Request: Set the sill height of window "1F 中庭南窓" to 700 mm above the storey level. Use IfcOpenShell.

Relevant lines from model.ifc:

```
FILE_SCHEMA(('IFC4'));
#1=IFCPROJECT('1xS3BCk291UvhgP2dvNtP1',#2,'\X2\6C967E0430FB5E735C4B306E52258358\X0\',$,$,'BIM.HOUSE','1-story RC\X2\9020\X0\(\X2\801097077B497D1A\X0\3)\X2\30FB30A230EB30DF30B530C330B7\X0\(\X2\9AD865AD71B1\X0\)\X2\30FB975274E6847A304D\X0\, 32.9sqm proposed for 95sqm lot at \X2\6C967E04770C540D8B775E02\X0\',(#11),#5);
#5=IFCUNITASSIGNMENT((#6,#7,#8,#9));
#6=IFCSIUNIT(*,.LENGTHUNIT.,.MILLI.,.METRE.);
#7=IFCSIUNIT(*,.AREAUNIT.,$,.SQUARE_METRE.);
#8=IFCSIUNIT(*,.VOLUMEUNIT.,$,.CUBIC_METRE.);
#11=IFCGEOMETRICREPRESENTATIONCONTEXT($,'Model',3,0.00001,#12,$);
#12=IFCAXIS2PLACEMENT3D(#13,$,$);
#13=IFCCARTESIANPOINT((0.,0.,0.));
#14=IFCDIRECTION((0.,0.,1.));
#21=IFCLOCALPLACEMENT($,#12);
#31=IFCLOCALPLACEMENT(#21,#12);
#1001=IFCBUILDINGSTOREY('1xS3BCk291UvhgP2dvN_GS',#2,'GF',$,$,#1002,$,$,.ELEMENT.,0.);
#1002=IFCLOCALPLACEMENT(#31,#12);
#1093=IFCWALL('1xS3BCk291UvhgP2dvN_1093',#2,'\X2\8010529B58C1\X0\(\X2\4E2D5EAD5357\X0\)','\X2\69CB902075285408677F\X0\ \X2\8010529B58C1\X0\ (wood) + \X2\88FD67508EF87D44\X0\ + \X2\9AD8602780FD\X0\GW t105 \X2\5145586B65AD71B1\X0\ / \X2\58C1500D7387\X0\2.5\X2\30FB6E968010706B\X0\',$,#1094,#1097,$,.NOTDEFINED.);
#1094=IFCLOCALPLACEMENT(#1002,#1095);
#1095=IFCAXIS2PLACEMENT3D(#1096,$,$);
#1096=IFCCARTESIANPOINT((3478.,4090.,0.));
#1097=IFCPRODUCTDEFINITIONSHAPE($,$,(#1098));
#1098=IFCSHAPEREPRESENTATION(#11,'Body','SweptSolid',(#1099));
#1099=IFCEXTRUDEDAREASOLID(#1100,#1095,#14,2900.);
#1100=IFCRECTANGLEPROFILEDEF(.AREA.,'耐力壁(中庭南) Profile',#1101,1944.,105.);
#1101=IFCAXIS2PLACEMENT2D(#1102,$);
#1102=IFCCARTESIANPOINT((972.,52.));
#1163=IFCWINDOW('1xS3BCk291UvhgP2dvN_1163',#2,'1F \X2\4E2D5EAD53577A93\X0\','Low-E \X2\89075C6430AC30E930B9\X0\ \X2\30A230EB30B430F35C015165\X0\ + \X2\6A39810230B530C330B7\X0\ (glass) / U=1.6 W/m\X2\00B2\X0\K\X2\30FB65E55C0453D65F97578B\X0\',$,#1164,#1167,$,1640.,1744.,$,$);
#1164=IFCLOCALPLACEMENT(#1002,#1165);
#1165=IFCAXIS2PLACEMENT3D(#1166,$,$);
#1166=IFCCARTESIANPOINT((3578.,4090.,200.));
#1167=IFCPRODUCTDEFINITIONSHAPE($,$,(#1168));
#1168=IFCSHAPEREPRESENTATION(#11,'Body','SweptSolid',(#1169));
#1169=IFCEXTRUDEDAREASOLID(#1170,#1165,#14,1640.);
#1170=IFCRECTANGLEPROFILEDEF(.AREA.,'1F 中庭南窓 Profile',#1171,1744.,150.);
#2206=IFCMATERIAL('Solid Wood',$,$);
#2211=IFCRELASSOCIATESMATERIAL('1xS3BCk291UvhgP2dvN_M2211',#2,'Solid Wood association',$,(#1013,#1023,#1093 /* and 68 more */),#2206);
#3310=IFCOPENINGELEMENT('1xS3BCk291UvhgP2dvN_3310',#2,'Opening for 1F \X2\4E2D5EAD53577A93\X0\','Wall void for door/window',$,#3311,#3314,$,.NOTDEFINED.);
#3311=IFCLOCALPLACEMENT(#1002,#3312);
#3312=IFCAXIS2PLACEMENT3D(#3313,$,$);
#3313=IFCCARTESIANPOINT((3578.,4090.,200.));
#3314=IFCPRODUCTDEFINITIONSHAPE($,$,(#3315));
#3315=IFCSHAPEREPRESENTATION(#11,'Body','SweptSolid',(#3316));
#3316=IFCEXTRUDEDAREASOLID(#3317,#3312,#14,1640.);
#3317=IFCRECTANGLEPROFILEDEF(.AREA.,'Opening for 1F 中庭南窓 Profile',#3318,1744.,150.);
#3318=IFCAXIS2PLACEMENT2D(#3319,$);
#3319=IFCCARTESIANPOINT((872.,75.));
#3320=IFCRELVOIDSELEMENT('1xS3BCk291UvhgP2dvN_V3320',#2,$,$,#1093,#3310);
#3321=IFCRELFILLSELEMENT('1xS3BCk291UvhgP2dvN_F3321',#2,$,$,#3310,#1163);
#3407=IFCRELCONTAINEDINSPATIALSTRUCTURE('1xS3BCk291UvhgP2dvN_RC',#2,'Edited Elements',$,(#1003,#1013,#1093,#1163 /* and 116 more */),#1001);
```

```python
import numpy as np
import ifcopenshell
import ifcopenshell.api.geometry
import ifcopenshell.geom
import ifcopenshell.util.element
import ifcopenshell.util.placement
import ifcopenshell.util.shape
import ifcopenshell.util.unit

model = ifcopenshell.open("model.ifc")
unit_scale = ifcopenshell.util.unit.calculate_unit_scale(model)

window = model.by_guid("1xS3BCk291UvhgP2dvN_1163")
opening = window.FillsVoids[0].RelatingOpeningElement
storey = ifcopenshell.util.element.get_container(window, ifc_class="IfcBuildingStorey")
level = ifcopenshell.util.placement.get_local_placement(storey.ObjectPlacement)[2, 3]

# The opening's origin need not be at the sill, so measure its lowest point.
shape = ifcopenshell.geom.create_shape(ifcopenshell.geom.settings(), opening)
bottom = ifcopenshell.util.shape.get_shape_bottom_elevation(shape, shape.geometry) / unit_scale
dz = level + 700.0 - bottom

shift = np.array([0.0, 0.0, dz])
# The window is not placed relative to its opening, so move both.
for product in (opening, window):
    matrix = ifcopenshell.util.placement.get_local_placement(product.ObjectPlacement)
    matrix[:3, 3] += shift
    ifcopenshell.api.geometry.edit_object_placement(model, product=product, matrix=matrix, is_si=False)

print(f"moved by {dz * unit_scale:+.3f} m")

model.write("model_updated.ifc")
```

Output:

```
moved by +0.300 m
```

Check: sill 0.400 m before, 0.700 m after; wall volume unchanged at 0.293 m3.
